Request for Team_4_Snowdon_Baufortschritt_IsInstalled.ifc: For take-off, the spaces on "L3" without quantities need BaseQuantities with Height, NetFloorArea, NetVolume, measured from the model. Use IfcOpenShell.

First a look at what the model holds.

```python
import ifcopenshell
import ifcopenshell.util.element
import ifcopenshell.util.unit

model = ifcopenshell.open("Team_4_Snowdon_Baufortschritt_IsInstalled.ifc")
print(model.schema)
for unit_type in ("LENGTHUNIT", "AREAUNIT", "VOLUMEUNIT"):
    print(unit_type, ifcopenshell.util.unit.calculate_unit_scale(model, unit_type))
storey = next(s for s in model.by_type("IfcBuildingStorey") if s.Name == "L3")
spaces = [e for e in ifcopenshell.util.element.get_decomposition(storey) if e.is_a("IfcSpace")]
for e in sorted(spaces, key=lambda e: e.id()):
    print(e.id(), e.is_a(), e.Name, list(ifcopenshell.util.element.get_psets(e, qtos_only=True)), sep=" | ")
```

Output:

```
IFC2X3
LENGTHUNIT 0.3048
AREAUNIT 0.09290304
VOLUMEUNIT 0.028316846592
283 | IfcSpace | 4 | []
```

```python
import ifcopenshell
import ifcopenshell.api.pset
import ifcopenshell.geom
import ifcopenshell.util.element
import ifcopenshell.util.shape
import ifcopenshell.util.unit

model = ifcopenshell.open("Team_4_Snowdon_Baufortschritt_IsInstalled.ifc")
unit_scale = ifcopenshell.util.unit.calculate_unit_scale(model)
area_scale = ifcopenshell.util.unit.calculate_unit_scale(model, "AREAUNIT")
volume_scale = ifcopenshell.util.unit.calculate_unit_scale(model, "VOLUMEUNIT")
settings = ifcopenshell.geom.settings()

storey = next(s for s in model.by_type("IfcBuildingStorey") if s.Name == "L3")
spaces = [e for e in ifcopenshell.util.element.get_decomposition(storey) if e.is_a("IfcSpace")]

for e in sorted(spaces, key=lambda e: e.id()):
    if ifcopenshell.util.element.get_psets(e, qtos_only=True, should_inherit=False):
        continue
    # Geometry comes back in metres, in the element's own axes.
    shape = ifcopenshell.geom.create_shape(settings, e)
    values = {
        "Height": ifcopenshell.util.shape.get_z(shape.geometry) / unit_scale,
        "NetFloorArea": ifcopenshell.util.shape.get_footprint_area(shape.geometry) / area_scale,
        "NetVolume": ifcopenshell.util.shape.get_volume(shape.geometry) / volume_scale,
    }
    qto = ifcopenshell.api.pset.add_qto(model, product=e, name="BaseQuantities")
    ifcopenshell.api.pset.edit_qto(model, qto=qto, properties=values)
    print(e.id(), {k: round(v, 3) for k, v in values.items()})

model.write("Team_4_Snowdon_Baufortschritt_IsInstalled_edited.ifc")
```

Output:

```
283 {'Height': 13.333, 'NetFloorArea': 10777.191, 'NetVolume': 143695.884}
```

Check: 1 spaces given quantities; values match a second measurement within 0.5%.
